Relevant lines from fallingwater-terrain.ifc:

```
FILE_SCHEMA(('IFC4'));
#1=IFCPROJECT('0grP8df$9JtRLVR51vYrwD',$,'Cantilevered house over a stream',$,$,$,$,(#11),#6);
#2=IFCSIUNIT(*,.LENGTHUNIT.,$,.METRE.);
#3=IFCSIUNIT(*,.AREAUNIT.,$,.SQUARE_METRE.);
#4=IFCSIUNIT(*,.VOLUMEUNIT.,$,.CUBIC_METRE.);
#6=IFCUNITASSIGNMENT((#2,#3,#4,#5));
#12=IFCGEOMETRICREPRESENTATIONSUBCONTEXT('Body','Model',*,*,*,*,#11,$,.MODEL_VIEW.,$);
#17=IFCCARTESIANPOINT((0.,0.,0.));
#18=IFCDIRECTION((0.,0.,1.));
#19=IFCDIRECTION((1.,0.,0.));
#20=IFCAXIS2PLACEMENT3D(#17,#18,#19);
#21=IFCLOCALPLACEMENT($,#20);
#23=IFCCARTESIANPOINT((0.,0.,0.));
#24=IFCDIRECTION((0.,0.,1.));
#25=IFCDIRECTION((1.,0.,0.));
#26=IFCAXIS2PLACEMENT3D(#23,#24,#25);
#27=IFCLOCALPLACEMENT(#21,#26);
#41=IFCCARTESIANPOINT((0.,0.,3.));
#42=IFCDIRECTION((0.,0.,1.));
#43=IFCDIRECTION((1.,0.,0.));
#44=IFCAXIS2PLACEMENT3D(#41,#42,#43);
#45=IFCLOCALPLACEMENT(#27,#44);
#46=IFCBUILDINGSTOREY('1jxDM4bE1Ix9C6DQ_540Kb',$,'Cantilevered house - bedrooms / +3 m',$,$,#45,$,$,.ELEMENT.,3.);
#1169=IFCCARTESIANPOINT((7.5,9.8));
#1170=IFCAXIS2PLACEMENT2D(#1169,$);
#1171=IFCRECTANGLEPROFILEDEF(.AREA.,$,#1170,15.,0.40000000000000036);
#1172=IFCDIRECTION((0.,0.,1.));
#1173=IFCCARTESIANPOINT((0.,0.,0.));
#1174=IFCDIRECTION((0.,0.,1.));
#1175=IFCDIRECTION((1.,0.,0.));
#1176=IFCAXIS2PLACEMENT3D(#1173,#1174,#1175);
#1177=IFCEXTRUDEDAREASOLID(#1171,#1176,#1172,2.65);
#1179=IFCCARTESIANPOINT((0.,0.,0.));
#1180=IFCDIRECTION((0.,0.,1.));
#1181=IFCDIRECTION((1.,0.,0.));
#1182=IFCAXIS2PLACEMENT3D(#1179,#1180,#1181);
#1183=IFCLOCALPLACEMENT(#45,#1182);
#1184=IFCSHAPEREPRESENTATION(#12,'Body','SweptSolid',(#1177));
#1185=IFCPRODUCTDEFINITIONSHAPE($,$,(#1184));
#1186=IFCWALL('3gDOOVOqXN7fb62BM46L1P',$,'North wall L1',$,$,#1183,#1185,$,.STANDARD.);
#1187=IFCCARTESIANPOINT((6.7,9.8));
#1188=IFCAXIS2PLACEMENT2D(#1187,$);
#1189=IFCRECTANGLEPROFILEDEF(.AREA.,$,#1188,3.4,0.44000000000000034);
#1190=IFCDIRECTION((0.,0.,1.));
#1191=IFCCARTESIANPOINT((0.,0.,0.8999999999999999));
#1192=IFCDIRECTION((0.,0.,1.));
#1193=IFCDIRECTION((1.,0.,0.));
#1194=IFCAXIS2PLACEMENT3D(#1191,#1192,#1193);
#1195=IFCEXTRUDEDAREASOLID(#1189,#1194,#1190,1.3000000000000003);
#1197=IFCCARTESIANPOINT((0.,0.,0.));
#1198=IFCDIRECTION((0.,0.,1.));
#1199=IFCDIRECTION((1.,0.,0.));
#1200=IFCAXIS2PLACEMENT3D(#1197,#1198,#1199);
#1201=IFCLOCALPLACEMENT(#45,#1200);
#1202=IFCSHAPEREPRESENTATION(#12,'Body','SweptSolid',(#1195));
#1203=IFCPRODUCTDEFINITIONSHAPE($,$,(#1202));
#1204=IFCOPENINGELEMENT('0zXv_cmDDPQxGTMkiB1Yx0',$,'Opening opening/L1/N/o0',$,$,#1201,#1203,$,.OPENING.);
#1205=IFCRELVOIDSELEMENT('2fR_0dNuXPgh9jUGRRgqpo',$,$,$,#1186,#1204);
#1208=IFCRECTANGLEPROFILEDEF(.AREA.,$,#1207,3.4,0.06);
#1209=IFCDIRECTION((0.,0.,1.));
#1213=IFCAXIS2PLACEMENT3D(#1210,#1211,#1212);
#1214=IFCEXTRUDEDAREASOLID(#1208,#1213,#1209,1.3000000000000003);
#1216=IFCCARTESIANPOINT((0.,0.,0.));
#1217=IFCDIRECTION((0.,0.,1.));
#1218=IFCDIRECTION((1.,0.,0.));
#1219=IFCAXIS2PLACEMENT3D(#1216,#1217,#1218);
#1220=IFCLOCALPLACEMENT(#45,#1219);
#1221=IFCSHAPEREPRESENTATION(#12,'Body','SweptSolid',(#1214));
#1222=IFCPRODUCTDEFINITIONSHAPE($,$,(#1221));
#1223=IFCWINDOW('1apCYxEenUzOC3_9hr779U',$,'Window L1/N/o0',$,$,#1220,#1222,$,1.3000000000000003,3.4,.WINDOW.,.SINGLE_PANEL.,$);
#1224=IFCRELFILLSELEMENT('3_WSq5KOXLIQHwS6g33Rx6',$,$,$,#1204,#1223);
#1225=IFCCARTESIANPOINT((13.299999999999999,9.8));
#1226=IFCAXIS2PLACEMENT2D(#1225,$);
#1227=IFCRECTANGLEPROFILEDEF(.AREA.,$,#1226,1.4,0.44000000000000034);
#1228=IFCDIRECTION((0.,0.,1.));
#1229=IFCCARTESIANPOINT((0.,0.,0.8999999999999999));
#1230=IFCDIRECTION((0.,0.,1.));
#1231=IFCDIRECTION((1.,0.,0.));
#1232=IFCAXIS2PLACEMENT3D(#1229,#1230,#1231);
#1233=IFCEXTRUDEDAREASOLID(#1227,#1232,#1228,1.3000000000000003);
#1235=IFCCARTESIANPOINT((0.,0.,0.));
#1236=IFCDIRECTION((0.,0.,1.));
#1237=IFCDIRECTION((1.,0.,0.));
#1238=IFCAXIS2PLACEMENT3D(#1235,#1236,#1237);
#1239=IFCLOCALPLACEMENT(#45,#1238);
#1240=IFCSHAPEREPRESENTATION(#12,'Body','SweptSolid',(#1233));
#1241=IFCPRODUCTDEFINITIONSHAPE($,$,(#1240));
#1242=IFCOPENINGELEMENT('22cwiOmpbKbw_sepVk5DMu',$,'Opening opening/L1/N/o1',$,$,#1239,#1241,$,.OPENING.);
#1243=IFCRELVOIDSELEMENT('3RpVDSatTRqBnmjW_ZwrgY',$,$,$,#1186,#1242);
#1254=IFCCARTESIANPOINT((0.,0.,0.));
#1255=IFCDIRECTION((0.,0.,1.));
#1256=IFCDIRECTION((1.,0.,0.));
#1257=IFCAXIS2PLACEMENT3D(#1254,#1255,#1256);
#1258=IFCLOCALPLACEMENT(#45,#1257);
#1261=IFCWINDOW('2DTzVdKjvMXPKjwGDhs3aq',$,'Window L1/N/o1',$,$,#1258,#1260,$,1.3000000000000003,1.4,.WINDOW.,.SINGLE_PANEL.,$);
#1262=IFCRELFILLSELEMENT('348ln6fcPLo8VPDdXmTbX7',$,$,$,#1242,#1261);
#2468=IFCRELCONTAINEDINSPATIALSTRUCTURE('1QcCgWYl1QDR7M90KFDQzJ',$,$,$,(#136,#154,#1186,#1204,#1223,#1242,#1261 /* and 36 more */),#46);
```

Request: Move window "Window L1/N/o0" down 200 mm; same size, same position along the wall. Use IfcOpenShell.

```python
import numpy as np
import ifcopenshell
import ifcopenshell.api.geometry
import ifcopenshell.util.placement
import ifcopenshell.util.unit

model = ifcopenshell.open("fallingwater-terrain.ifc")
unit_scale = ifcopenshell.util.unit.calculate_unit_scale(model)

window = model.by_guid("1apCYxEenUzOC3_9hr779U")
opening = window.FillsVoids[0].RelatingOpeningElement
dz = -0.2 / unit_scale

shift = np.array([0.0, 0.0, dz])
# The window is not placed relative to its opening, so move both.
for product in (opening, window):
    matrix = ifcopenshell.util.placement.get_local_placement(product.ObjectPlacement)
    matrix[:3, 3] += shift
    ifcopenshell.api.geometry.edit_object_placement(model, product=product, matrix=matrix, is_si=False)

print(f"moved by {dz * unit_scale:+.3f} m")

model.write("fallingwater-terrain_edited.ifc")
```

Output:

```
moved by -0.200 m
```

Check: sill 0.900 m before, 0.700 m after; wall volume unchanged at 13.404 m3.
